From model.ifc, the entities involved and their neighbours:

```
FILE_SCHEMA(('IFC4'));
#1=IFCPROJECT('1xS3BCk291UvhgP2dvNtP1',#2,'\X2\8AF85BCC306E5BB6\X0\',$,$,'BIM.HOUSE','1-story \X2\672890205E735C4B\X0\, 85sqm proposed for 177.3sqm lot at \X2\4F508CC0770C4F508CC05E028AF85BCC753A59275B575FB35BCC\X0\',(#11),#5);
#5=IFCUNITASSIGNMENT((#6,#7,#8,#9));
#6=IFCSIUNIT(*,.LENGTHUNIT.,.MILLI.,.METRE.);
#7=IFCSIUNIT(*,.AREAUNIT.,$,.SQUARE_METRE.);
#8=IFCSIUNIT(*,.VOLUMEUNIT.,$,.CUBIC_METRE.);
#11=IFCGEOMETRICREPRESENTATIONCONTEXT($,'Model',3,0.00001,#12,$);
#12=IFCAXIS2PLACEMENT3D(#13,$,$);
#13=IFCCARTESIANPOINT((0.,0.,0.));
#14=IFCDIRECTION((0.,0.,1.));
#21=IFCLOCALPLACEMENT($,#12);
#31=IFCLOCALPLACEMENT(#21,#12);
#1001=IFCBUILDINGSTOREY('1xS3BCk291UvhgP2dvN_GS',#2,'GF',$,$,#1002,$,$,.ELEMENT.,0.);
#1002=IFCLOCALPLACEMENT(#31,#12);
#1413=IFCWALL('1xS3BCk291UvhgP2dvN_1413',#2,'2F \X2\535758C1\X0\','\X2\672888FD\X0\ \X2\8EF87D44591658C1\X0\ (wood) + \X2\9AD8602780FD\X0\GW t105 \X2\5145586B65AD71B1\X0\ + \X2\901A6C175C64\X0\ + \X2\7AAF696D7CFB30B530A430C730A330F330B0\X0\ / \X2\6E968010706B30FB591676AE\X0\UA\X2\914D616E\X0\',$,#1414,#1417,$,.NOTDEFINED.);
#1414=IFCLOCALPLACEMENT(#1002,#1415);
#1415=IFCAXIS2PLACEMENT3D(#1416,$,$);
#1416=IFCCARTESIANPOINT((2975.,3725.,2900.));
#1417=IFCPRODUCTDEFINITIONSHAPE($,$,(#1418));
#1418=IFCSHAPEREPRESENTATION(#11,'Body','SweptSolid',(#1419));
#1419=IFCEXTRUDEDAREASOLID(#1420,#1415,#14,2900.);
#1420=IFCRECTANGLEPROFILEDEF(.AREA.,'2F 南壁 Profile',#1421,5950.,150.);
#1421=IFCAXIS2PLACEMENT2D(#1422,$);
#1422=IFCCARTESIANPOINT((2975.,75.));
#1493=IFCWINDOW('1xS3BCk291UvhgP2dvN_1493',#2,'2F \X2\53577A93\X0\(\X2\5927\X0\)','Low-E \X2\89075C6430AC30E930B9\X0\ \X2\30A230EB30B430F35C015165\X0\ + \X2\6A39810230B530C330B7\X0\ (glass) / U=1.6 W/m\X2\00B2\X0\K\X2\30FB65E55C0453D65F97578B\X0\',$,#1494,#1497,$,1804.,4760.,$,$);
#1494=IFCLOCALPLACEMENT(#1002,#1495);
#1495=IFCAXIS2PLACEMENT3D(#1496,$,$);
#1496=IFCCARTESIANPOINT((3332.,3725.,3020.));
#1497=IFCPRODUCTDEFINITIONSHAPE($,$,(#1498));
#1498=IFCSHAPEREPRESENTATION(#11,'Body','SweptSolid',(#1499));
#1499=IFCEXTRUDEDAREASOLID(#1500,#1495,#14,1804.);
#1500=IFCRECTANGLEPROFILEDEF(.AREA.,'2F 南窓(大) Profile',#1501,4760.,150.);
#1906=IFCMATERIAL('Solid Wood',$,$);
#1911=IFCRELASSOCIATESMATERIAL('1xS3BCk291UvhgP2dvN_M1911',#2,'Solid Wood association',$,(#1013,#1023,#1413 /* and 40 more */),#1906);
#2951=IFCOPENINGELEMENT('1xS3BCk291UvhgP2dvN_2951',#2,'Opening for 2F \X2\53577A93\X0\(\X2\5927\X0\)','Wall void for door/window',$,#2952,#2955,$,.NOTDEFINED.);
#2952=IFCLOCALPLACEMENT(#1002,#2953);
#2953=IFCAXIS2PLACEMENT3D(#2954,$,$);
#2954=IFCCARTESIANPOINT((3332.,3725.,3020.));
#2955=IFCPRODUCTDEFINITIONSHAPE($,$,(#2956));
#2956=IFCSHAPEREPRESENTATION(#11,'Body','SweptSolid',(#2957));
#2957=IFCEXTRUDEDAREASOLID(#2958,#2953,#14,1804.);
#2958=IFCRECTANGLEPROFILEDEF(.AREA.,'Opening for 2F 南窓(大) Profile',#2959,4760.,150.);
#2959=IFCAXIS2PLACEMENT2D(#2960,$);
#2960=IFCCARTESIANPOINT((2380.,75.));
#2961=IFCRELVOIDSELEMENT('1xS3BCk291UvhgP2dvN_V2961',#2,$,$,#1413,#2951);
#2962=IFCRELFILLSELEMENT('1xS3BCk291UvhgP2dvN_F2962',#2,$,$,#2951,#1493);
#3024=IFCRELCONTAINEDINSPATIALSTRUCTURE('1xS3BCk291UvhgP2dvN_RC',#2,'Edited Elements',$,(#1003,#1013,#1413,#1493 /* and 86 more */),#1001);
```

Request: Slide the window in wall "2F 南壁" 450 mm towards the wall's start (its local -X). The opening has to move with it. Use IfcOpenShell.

```python
import ifcopenshell
import ifcopenshell.api.geometry
import ifcopenshell.util.placement
import ifcopenshell.util.unit

model = ifcopenshell.open("model.ifc")
unit_scale = ifcopenshell.util.unit.calculate_unit_scale(model)

window = model.by_guid("1xS3BCk291UvhgP2dvN_1493")
opening = window.FillsVoids[0].RelatingOpeningElement
wall = opening.VoidsElements[0].RelatingBuildingElement

wall_matrix = ifcopenshell.util.placement.get_local_placement(wall.ObjectPlacement)
shift = wall_matrix[:3, 0] * -0.45 / unit_scale
before = ifcopenshell.util.placement.get_local_placement(window.ObjectPlacement)[:3, 3].copy()

# The window is not placed relative to its opening, so move both.
for product in (opening, window):
    matrix = ifcopenshell.util.placement.get_local_placement(product.ObjectPlacement)
    matrix[:3, 3] += shift
    ifcopenshell.api.geometry.edit_object_placement(model, product=product, matrix=matrix, is_si=False)

after = ifcopenshell.util.placement.get_local_placement(window.ObjectPlacement)[:3, 3]
print("window moved by", (after - before).round(3) + 0.0)

model.write("model_v2.ifc")
```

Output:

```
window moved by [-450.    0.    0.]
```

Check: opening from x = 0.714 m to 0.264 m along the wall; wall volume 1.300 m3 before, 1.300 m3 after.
